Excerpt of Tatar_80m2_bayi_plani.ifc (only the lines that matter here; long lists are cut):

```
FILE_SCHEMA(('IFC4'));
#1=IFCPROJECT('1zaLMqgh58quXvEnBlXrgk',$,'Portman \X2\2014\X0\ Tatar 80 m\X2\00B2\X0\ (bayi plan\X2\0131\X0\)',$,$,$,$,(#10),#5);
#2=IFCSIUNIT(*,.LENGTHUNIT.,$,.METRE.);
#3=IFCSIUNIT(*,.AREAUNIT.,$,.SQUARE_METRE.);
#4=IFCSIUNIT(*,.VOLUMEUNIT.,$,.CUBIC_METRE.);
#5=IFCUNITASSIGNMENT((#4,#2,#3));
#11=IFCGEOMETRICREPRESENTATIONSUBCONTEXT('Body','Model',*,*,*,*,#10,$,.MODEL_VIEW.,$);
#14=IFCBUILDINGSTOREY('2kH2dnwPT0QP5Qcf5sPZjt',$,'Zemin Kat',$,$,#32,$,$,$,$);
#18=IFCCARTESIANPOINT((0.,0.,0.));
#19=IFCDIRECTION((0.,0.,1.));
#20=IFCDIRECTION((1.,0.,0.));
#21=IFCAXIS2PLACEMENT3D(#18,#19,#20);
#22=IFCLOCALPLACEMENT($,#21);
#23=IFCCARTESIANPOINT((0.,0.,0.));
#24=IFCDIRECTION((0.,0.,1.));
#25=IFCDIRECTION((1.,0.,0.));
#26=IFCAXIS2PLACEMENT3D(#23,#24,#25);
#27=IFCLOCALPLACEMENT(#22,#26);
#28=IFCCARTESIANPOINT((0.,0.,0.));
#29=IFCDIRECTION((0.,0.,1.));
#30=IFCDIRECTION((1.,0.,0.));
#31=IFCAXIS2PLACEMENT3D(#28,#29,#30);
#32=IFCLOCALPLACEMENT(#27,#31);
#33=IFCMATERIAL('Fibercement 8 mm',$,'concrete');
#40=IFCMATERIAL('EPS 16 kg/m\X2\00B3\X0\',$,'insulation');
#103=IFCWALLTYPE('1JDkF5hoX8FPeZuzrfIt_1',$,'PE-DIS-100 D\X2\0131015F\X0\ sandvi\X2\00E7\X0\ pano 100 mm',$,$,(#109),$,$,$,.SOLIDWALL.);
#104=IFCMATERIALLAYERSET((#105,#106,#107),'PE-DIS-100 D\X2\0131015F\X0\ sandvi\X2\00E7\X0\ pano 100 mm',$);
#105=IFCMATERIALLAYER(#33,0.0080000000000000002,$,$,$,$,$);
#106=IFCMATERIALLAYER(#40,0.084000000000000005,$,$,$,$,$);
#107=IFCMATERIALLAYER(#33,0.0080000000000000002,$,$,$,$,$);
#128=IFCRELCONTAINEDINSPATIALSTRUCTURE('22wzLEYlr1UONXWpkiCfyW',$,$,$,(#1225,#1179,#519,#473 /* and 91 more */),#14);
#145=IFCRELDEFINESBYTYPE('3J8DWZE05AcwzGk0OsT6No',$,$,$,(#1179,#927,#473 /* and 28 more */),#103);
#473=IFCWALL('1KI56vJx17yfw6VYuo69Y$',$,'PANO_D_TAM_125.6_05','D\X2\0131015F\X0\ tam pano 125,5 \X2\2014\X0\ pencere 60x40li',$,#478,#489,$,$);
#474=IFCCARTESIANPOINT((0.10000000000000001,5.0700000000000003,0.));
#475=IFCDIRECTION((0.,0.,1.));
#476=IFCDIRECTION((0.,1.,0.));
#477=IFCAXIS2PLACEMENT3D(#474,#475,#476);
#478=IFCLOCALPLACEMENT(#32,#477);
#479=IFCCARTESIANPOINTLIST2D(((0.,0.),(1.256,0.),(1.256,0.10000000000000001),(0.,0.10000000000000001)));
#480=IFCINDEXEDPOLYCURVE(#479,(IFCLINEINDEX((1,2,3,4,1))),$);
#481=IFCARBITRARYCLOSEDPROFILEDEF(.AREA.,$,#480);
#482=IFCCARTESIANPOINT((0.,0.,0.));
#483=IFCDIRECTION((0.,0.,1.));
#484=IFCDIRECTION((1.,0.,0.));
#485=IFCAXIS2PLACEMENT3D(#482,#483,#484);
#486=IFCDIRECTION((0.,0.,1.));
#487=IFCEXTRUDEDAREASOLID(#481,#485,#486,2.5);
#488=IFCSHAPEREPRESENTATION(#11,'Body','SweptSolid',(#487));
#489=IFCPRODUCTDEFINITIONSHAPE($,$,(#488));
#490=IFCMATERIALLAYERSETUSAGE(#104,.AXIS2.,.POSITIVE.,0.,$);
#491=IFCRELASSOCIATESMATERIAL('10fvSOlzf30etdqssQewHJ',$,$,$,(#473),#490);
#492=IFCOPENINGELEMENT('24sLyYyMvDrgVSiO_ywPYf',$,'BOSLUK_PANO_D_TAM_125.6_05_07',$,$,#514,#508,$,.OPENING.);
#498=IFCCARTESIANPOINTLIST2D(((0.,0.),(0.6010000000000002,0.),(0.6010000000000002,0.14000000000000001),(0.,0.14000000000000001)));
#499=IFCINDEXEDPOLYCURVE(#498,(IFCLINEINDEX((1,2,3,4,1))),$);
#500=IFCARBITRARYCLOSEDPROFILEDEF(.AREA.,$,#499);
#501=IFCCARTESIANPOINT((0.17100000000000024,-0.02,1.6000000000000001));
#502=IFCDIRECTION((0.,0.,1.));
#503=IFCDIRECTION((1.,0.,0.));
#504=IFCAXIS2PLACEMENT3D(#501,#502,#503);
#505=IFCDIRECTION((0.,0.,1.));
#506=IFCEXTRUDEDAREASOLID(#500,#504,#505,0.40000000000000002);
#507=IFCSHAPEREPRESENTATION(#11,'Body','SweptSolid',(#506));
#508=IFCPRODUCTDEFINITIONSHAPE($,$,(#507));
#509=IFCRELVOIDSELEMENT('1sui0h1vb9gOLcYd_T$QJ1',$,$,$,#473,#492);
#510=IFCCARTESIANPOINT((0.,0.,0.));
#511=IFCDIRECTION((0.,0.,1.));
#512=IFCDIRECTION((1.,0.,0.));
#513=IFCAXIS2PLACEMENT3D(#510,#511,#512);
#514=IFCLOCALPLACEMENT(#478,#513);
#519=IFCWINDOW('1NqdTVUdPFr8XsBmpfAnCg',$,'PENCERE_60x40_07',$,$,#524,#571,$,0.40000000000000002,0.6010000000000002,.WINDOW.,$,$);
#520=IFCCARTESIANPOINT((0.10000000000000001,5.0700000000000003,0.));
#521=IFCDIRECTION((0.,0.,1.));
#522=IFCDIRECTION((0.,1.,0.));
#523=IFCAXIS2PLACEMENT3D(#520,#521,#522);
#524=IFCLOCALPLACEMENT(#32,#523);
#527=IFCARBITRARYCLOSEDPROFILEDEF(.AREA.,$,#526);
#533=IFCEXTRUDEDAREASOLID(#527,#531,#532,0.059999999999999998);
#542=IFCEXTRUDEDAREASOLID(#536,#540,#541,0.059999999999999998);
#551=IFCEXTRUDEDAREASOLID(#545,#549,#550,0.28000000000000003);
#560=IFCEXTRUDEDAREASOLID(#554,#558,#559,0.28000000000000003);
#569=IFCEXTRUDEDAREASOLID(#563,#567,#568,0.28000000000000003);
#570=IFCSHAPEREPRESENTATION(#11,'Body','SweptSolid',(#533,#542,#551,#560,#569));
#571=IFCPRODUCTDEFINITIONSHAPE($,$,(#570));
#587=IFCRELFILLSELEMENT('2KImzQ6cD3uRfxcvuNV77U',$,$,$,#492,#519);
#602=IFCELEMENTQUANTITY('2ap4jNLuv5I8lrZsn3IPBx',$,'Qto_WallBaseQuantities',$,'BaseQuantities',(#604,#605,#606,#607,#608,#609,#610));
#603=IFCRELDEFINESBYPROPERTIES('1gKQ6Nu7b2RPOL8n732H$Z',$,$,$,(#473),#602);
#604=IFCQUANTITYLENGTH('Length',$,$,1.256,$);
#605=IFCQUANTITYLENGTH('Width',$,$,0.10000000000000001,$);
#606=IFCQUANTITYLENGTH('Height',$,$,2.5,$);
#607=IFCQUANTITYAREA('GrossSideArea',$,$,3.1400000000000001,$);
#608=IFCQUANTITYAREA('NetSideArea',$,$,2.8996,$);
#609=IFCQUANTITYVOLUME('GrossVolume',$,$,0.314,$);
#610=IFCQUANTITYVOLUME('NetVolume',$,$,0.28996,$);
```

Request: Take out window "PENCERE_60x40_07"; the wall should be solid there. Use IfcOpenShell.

```python
import ifcopenshell
import ifcopenshell.api.feature
import ifcopenshell.api.pset
import ifcopenshell.api.root
import ifcopenshell.geom
import ifcopenshell.util.element
import ifcopenshell.util.shape
import ifcopenshell.util.unit

model = ifcopenshell.open("Tatar_80m2_bayi_plani.ifc")
area_scale = ifcopenshell.util.unit.calculate_unit_scale(model, "AREAUNIT")
volume_scale = ifcopenshell.util.unit.calculate_unit_scale(model, "VOLUMEUNIT")
settings = ifcopenshell.geom.settings()


def volume(element):
    """Net volume in cubic metres, openings subtracted."""
    shape = ifcopenshell.geom.create_shape(settings, element)
    return ifcopenshell.util.shape.get_volume(shape.geometry)


window = model.by_guid("1NqdTVUdPFr8XsBmpfAnCg")
opening = window.FillsVoids[0].RelatingOpeningElement
wall = opening.VoidsElements[0].RelatingBuildingElement
before = volume(wall)

ifcopenshell.api.root.remove_product(model, product=window)
ifcopenshell.api.feature.remove_feature(model, feature=opening)

after = volume(wall)
thickness = 0.1  # wall thickness in metres

# Update the wall's stored quantities.
qto = model.by_id(ifcopenshell.util.element.get_pset(wall, "Qto_WallBaseQuantities", should_inherit=False)["id"])
ifcopenshell.api.pset.edit_qto(model, qto=qto, properties={
    "NetSideArea": after / thickness / area_scale,
    "NetVolume": after / volume_scale,
})

print(f"wall volume {before:.3f} -> {after:.3f} m3")

model.write("Tatar_80m2_bayi_plani_rev.ifc")
```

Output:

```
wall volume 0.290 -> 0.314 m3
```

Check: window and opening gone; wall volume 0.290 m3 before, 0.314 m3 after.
